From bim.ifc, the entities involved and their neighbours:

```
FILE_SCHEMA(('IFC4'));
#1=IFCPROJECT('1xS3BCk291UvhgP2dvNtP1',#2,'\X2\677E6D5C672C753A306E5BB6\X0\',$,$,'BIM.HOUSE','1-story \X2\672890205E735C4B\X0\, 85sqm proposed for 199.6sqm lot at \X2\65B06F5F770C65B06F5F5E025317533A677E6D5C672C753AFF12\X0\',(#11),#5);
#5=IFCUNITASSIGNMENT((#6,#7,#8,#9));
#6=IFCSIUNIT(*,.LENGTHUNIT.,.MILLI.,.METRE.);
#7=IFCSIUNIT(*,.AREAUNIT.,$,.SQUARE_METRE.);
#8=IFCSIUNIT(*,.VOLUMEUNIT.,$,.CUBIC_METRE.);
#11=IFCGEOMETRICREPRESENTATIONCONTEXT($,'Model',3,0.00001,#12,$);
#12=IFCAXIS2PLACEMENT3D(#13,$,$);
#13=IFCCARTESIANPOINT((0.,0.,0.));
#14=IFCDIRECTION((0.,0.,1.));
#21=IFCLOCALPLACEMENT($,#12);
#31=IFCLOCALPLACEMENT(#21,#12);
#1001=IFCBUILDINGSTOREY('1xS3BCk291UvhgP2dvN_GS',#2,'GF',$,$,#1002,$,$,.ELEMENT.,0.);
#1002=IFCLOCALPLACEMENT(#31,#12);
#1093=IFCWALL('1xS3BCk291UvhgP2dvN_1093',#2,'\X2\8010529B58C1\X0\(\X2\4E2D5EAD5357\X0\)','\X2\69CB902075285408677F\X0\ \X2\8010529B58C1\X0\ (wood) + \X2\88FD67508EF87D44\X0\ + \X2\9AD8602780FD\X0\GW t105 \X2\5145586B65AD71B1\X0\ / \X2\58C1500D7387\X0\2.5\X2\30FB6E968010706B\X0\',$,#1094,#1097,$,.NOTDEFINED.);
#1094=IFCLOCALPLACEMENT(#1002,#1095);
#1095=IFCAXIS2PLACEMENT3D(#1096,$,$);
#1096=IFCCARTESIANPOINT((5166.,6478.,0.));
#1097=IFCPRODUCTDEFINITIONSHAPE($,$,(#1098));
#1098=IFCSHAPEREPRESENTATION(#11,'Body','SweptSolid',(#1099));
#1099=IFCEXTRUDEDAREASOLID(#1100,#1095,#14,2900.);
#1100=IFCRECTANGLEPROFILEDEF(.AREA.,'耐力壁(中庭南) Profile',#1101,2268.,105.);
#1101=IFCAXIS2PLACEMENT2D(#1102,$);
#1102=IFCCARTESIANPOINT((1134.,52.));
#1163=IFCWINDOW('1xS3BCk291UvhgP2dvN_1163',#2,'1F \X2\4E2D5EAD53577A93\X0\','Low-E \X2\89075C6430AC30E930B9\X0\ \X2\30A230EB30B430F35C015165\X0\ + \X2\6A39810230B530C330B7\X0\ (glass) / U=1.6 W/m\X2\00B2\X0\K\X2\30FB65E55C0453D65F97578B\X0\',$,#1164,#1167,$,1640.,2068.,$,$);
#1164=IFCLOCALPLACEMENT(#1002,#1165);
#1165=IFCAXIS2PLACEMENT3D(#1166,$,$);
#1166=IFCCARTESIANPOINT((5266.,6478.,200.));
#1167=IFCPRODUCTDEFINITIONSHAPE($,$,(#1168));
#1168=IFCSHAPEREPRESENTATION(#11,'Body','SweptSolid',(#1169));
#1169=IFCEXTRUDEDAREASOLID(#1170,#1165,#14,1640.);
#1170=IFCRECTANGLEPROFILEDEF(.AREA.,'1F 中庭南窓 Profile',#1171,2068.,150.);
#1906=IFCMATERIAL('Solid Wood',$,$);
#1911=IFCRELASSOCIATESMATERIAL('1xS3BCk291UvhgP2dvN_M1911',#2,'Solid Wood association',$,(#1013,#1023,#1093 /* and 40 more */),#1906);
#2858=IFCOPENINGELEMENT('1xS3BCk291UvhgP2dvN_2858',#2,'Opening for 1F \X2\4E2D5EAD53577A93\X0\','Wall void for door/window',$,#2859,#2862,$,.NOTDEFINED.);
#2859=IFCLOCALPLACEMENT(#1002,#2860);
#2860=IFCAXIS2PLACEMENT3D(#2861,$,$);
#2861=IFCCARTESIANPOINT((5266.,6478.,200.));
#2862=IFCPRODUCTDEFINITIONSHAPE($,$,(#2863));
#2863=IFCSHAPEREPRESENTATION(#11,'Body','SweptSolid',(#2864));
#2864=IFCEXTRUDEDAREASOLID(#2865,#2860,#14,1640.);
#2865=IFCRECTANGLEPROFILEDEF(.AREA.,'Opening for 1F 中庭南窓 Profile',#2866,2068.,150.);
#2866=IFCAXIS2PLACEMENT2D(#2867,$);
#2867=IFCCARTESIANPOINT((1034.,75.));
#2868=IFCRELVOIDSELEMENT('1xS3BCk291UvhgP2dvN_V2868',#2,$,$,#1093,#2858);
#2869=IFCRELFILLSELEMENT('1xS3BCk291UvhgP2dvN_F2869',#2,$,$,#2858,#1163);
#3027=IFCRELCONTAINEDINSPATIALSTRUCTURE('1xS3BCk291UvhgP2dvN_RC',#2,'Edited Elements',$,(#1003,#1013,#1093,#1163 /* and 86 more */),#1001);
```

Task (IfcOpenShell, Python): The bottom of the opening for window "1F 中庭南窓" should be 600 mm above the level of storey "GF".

```python
import numpy as np
import ifcopenshell
import ifcopenshell.api.geometry
import ifcopenshell.geom
import ifcopenshell.util.element
import ifcopenshell.util.placement
import ifcopenshell.util.shape
import ifcopenshell.util.unit

model = ifcopenshell.open("bim.ifc")
unit_scale = ifcopenshell.util.unit.calculate_unit_scale(model)

window = model.by_guid("1xS3BCk291UvhgP2dvN_1163")
opening = window.FillsVoids[0].RelatingOpeningElement
storey = ifcopenshell.util.element.get_container(window, ifc_class="IfcBuildingStorey")
level = ifcopenshell.util.placement.get_local_placement(storey.ObjectPlacement)[2, 3]

# The opening's origin need not be at the sill, so measure its lowest point.
shape = ifcopenshell.geom.create_shape(ifcopenshell.geom.settings(), opening)
bottom = ifcopenshell.util.shape.get_shape_bottom_elevation(shape, shape.geometry) / unit_scale
dz = level + 600.0 - bottom

shift = np.array([0.0, 0.0, dz])
# The window is not placed relative to its opening, so move both.
for product in (opening, window):
    matrix = ifcopenshell.util.placement.get_local_placement(product.ObjectPlacement)
    matrix[:3, 3] += shift
    ifcopenshell.api.geometry.edit_object_placement(model, product=product, matrix=matrix, is_si=False)

print(f"moved by {dz * unit_scale:+.3f} m")

model.write("bim_v2.ifc")
```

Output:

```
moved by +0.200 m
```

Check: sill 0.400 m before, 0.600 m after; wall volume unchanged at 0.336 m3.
